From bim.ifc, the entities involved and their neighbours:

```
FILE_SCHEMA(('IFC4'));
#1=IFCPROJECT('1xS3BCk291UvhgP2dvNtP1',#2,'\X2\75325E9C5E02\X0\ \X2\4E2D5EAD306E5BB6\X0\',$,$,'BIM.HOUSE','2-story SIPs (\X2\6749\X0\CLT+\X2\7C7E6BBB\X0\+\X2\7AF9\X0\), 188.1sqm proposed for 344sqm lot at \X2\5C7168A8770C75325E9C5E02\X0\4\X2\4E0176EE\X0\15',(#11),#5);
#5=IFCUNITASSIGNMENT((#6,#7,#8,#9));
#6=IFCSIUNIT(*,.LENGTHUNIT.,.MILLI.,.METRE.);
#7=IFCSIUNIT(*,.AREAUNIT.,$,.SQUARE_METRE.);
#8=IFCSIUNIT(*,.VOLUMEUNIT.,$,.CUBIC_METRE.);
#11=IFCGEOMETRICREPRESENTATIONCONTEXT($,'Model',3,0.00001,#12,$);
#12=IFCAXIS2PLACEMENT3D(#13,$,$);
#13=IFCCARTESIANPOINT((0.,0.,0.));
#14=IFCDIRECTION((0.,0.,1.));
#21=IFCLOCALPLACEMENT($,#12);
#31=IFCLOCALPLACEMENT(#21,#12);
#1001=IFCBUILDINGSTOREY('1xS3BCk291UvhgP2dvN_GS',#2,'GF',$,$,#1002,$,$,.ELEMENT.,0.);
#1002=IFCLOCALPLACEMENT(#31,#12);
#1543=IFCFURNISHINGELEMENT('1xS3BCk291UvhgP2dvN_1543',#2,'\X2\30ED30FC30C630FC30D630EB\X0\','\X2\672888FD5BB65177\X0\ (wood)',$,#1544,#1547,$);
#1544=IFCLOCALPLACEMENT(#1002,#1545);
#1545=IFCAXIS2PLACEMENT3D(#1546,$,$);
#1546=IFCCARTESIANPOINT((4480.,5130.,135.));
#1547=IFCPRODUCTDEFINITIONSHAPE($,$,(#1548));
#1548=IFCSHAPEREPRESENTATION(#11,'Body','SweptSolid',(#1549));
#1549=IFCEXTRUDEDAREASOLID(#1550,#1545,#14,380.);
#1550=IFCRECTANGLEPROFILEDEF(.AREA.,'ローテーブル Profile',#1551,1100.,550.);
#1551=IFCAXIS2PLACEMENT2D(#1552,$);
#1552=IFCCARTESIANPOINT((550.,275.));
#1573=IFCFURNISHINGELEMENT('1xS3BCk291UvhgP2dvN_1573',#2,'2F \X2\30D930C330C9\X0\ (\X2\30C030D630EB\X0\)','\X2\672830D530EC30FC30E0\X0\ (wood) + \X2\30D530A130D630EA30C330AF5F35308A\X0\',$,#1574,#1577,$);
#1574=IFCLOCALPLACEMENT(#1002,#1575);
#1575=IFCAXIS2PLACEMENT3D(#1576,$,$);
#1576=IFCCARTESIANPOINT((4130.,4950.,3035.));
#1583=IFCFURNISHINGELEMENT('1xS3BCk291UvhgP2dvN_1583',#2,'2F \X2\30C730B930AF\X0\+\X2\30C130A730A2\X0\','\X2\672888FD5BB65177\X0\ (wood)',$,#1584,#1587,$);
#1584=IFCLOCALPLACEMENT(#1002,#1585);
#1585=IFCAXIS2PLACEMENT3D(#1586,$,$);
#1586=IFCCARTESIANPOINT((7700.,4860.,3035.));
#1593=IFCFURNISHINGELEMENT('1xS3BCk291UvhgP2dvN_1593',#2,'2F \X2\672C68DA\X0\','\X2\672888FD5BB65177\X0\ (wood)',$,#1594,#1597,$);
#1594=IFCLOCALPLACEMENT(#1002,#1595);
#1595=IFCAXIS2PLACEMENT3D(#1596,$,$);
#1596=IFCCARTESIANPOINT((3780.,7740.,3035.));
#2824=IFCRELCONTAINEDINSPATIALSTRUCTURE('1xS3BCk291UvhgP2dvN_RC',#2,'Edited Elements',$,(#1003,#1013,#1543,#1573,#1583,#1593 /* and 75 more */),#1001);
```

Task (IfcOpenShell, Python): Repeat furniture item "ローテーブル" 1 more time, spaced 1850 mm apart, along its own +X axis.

```python
import ifcopenshell
import ifcopenshell.api.geometry
import ifcopenshell.api.root
import ifcopenshell.util.element
import ifcopenshell.util.placement
import ifcopenshell.util.unit

model = ifcopenshell.open("bim.ifc")
unit_scale = ifcopenshell.util.unit.calculate_unit_scale(model)


def reuse_history(source, copy):
    """copy_class also copies each property set's owner history, people and application; keep the originals."""
    for rel in copy.IsDefinedBy:
        if rel.is_a("IfcRelDefinesByProperties") and (history := rel.RelatingPropertyDefinition.OwnerHistory):
            rel.RelatingPropertyDefinition.OwnerHistory = source.OwnerHistory
            ifcopenshell.util.element.remove_deep2(model, history)


source = model.by_id(1543)
base = ifcopenshell.util.placement.get_local_placement(source.ObjectPlacement)
step = base[:3, 0] * 1.85 / unit_scale

for i in range(1, 2):
    copy = ifcopenshell.api.root.copy_class(model, product=source)
    copy.Representation = ifcopenshell.util.element.copy_deep(
        model, source.Representation, exclude=["IfcGeometricRepresentationContext", "IfcRepresentationMap"]
    )
    reuse_history(source, copy)
    matrix = base.copy()
    matrix[:3, 3] += i * step
    print("added at", matrix[:3, 3].round(3) + 0.0)
    ifcopenshell.api.geometry.edit_object_placement(model, product=copy, matrix=matrix, is_si=False)

model.write("bim_v2.ifc")
```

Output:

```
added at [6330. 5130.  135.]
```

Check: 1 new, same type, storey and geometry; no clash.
